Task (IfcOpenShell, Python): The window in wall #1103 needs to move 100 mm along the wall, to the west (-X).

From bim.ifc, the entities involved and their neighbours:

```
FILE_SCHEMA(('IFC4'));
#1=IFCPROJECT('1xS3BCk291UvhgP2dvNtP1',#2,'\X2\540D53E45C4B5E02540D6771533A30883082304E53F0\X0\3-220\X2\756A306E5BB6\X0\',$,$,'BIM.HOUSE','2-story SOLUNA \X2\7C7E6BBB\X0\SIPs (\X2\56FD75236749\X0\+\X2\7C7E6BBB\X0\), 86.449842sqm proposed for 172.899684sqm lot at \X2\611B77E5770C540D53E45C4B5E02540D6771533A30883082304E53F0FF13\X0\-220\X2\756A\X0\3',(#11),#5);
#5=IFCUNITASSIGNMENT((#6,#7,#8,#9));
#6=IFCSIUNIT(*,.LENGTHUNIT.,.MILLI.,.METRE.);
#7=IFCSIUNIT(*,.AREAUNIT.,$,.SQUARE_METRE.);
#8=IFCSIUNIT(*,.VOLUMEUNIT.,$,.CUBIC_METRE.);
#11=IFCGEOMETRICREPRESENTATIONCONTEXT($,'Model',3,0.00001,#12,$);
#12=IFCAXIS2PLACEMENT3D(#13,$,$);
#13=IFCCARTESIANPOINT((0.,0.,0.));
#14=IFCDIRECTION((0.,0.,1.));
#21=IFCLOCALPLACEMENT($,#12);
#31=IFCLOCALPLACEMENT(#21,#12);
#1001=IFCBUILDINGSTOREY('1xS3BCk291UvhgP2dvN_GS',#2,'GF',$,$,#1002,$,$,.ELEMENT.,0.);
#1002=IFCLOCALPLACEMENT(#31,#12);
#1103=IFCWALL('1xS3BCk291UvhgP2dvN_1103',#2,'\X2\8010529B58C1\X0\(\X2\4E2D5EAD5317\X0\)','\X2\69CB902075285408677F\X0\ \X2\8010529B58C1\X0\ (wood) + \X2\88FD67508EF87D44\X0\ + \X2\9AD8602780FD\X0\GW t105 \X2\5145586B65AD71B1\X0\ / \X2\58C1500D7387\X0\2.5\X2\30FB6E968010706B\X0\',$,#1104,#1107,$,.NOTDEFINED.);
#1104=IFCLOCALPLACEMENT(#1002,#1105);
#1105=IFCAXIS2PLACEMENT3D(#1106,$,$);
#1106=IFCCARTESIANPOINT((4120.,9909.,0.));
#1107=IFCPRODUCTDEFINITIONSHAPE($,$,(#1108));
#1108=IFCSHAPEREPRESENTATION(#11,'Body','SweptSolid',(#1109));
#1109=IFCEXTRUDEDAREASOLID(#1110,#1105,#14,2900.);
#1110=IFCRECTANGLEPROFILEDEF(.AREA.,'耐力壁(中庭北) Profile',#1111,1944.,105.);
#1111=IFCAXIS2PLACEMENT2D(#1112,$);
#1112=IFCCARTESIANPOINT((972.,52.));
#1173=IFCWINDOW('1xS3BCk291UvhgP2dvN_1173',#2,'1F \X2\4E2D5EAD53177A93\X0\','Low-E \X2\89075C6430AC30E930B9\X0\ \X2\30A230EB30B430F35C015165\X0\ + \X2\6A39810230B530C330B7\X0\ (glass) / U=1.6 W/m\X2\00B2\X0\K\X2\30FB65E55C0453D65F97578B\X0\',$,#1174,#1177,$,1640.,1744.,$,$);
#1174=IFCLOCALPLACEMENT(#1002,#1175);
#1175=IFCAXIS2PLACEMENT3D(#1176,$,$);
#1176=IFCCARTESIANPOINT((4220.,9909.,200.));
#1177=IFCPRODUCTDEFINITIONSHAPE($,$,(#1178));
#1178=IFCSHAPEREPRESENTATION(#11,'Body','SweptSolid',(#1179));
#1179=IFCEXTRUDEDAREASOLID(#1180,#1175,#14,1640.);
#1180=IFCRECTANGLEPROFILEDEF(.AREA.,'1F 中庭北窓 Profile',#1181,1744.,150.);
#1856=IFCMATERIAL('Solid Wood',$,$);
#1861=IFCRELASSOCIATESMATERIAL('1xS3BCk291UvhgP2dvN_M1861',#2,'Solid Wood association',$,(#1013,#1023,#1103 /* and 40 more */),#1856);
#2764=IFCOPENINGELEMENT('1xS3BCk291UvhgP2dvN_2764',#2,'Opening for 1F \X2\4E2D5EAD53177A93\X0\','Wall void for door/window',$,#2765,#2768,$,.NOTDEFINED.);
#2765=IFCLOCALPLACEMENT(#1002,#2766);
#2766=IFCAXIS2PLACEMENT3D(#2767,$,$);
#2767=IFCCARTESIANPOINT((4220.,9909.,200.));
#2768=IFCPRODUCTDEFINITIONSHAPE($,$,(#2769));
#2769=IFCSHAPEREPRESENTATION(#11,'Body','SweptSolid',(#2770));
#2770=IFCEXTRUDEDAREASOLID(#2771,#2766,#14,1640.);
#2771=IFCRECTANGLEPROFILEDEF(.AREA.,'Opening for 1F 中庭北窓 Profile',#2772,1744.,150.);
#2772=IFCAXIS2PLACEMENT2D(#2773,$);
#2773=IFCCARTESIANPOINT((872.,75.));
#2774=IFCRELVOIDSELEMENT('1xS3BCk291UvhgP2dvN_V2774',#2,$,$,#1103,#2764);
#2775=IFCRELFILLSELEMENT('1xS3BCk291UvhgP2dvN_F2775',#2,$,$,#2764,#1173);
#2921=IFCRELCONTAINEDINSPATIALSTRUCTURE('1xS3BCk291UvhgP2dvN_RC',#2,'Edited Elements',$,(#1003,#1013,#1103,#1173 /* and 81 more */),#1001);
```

```python
import ifcopenshell
import ifcopenshell.api.geometry
import ifcopenshell.util.placement
import ifcopenshell.util.unit

model = ifcopenshell.open("bim.ifc")
unit_scale = ifcopenshell.util.unit.calculate_unit_scale(model)

window = model.by_guid("1xS3BCk291UvhgP2dvN_1173")
opening = window.FillsVoids[0].RelatingOpeningElement
wall = opening.VoidsElements[0].RelatingBuildingElement

wall_matrix = ifcopenshell.util.placement.get_local_placement(wall.ObjectPlacement)
shift = wall_matrix[:3, 0] * -0.1 / unit_scale
before = ifcopenshell.util.placement.get_local_placement(window.ObjectPlacement)[:3, 3].copy()

# The window is not placed relative to its opening, so move both.
for product in (opening, window):
    matrix = ifcopenshell.util.placement.get_local_placement(product.ObjectPlacement)
    matrix[:3, 3] += shift
    ifcopenshell.api.geometry.edit_object_placement(model, product=product, matrix=matrix, is_si=False)

after = ifcopenshell.util.placement.get_local_placement(window.ObjectPlacement)[:3, 3]
print("window moved by", (after - before).round(3) + 0.0)

model.write("bim-out.ifc")
```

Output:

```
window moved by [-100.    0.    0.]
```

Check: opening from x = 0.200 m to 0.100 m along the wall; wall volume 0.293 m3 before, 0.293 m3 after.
